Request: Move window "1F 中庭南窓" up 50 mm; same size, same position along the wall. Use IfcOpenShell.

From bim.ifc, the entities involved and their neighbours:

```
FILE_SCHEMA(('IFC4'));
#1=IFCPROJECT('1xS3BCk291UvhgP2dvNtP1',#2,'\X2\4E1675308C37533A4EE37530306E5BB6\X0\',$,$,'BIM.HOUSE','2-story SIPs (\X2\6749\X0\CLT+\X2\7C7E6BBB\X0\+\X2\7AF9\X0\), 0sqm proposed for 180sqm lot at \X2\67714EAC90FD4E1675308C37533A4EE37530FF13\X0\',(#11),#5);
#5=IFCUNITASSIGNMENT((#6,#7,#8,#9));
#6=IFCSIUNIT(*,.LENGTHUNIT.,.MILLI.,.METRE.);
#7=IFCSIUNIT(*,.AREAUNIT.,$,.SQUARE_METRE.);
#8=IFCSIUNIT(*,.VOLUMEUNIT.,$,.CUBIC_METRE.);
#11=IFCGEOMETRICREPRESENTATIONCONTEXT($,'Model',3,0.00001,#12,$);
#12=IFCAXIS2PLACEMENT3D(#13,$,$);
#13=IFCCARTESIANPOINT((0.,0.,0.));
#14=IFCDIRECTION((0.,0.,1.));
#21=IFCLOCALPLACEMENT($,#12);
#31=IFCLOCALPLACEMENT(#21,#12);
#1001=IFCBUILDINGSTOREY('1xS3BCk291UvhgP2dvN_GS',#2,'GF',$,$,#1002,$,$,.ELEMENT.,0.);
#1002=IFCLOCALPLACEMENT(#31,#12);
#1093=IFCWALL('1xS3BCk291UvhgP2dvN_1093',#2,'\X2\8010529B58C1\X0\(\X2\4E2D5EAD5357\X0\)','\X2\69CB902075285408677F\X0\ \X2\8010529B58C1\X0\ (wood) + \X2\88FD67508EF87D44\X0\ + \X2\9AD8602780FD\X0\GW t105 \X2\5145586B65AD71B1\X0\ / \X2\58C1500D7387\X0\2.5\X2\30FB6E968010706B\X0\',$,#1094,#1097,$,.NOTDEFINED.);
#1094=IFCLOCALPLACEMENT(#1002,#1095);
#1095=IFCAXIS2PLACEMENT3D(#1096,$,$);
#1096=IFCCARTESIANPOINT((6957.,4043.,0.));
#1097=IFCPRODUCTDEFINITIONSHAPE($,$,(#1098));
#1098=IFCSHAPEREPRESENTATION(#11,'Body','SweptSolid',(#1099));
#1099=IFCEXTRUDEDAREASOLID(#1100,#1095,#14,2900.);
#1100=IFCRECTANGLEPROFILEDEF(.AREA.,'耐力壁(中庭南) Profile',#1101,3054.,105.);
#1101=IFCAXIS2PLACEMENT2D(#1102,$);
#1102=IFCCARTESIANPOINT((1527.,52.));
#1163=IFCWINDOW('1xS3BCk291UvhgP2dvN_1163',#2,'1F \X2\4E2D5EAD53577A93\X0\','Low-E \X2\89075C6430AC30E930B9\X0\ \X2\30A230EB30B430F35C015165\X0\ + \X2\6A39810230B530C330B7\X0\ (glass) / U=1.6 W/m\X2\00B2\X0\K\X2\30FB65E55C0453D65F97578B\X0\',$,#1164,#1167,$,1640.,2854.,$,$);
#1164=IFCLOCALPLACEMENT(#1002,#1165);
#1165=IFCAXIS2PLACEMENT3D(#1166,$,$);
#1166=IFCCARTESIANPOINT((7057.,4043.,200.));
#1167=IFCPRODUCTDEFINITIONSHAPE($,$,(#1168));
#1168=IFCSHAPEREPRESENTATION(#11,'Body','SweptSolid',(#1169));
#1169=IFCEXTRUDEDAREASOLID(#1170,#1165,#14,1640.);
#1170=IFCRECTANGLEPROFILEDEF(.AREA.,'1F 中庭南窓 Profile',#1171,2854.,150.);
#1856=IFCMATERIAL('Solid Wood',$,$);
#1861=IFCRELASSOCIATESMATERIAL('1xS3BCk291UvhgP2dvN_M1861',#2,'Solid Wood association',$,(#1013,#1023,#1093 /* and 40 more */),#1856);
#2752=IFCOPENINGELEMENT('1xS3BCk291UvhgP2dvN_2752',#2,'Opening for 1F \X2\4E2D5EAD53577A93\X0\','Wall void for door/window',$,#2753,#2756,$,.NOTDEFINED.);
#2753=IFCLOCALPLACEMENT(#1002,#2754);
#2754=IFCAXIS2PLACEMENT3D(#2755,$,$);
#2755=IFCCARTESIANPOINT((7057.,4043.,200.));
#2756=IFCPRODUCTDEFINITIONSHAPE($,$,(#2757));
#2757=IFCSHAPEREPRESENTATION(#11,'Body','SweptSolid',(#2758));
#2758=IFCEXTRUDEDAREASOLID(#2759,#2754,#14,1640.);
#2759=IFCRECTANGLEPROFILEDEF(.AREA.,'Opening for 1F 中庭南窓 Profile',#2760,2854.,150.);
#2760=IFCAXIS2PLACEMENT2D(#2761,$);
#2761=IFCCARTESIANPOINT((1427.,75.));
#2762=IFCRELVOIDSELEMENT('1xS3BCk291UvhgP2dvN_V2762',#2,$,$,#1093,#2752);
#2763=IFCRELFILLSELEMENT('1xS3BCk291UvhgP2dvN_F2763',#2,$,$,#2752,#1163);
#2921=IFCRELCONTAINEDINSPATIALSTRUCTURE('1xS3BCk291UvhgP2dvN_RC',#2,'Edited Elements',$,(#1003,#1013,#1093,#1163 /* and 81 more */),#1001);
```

```python
import numpy as np
import ifcopenshell
import ifcopenshell.api.geometry
import ifcopenshell.util.placement
import ifcopenshell.util.unit

model = ifcopenshell.open("bim.ifc")
unit_scale = ifcopenshell.util.unit.calculate_unit_scale(model)

window = model.by_id(1163)
opening = window.FillsVoids[0].RelatingOpeningElement
dz = 0.05 / unit_scale

shift = np.array([0.0, 0.0, dz])
# The window is not placed relative to its opening, so move both.
for product in (opening, window):
    matrix = ifcopenshell.util.placement.get_local_placement(product.ObjectPlacement)
    matrix[:3, 3] += shift
    ifcopenshell.api.geometry.edit_object_placement(model, product=product, matrix=matrix, is_si=False)

print(f"moved by {dz * unit_scale:+.3f} m")

model.write("bim_updated.ifc")
```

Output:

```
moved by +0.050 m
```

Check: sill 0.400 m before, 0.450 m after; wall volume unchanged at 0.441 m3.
